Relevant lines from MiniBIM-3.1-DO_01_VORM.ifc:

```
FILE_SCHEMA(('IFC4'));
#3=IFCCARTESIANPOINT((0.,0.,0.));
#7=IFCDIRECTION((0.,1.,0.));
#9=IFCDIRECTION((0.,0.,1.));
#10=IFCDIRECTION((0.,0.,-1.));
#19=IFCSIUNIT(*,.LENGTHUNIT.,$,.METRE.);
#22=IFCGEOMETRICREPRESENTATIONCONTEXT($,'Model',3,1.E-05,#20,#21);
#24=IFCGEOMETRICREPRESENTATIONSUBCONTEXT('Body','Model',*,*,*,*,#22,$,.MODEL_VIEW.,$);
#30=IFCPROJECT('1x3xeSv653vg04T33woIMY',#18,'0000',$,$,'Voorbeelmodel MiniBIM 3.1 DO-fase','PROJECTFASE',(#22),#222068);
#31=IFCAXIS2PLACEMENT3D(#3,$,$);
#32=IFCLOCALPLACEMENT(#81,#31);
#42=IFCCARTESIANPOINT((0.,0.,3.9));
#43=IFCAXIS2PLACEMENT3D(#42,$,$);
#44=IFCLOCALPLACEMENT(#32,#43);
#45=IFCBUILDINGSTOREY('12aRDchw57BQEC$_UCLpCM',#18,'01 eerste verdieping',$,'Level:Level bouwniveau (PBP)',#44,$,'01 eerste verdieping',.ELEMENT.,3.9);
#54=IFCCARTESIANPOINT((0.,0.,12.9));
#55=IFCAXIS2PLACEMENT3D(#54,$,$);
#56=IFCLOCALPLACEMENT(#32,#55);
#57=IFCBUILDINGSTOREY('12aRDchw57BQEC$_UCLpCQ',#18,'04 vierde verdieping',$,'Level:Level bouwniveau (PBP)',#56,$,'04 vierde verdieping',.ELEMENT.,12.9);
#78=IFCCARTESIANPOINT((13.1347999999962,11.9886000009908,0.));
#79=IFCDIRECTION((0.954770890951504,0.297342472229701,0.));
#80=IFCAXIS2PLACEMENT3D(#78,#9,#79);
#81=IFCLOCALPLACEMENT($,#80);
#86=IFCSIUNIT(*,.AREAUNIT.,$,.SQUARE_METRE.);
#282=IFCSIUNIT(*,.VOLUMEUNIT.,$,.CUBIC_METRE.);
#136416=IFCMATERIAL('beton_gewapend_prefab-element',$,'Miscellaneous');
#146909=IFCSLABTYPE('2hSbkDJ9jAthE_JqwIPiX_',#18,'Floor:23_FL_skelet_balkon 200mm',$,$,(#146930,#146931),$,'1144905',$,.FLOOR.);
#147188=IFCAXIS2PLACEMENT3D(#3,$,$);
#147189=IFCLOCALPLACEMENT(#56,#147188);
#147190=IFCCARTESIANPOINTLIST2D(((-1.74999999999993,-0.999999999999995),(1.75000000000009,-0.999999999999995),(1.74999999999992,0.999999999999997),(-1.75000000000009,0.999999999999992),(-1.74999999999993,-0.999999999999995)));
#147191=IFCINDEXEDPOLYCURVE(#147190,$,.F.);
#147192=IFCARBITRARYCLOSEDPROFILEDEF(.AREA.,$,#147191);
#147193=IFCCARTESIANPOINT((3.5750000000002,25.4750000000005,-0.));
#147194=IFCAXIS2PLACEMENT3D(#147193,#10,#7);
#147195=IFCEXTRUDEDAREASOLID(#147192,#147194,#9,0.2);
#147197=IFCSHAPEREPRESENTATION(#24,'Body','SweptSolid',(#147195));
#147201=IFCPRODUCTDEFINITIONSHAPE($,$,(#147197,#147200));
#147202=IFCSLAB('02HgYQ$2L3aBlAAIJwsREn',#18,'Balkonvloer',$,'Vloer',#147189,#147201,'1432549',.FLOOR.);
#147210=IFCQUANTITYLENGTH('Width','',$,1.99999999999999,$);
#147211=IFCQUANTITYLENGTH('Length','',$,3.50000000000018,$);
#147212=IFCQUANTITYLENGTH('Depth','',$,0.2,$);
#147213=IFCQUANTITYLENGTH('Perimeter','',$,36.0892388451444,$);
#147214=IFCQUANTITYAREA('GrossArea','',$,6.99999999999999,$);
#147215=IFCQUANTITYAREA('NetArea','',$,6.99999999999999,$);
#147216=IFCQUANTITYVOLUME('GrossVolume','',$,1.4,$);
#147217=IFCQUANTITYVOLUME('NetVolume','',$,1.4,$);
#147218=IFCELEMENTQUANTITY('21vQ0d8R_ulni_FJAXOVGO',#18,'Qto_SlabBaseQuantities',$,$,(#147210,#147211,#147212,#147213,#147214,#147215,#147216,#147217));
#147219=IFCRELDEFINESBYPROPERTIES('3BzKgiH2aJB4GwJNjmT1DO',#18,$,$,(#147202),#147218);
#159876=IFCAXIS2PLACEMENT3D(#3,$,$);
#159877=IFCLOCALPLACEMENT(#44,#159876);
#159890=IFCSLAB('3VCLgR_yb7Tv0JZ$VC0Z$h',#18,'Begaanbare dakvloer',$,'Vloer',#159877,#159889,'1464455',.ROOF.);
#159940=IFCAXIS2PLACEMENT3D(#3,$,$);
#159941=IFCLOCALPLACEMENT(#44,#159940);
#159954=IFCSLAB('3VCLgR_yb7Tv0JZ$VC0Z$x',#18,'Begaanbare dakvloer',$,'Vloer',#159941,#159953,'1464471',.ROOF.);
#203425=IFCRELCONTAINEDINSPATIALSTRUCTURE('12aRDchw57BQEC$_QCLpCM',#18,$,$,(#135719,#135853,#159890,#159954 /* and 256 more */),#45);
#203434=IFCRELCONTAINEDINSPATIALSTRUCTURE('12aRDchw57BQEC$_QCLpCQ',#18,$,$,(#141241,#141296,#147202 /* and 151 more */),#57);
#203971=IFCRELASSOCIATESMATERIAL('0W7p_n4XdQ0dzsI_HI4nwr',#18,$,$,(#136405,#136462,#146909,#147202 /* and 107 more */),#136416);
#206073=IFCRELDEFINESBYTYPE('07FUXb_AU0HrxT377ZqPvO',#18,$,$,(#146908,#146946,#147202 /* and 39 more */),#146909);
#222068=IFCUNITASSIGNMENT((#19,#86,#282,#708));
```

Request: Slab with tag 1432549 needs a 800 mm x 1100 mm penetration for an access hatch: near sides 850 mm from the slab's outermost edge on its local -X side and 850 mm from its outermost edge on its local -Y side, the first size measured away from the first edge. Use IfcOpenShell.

```python
import numpy as np
import ifcopenshell
import ifcopenshell.api.feature
import ifcopenshell.api.geometry
import ifcopenshell.api.pset
import ifcopenshell.api.root
import ifcopenshell.geom
import ifcopenshell.util.element
import ifcopenshell.util.placement
import ifcopenshell.util.representation
import ifcopenshell.util.shape
import ifcopenshell.util.unit

model = ifcopenshell.open("MiniBIM-3.1-DO_01_VORM.ifc")
unit_scale = ifcopenshell.util.unit.calculate_unit_scale(model)
area_scale = ifcopenshell.util.unit.calculate_unit_scale(model, "AREAUNIT")
volume_scale = ifcopenshell.util.unit.calculate_unit_scale(model, "VOLUMEUNIT")
settings = ifcopenshell.geom.settings()


def volume(element):
    """Net volume in cubic metres, openings subtracted."""
    shape = ifcopenshell.geom.create_shape(settings, element)
    return ifcopenshell.util.shape.get_volume(shape.geometry)


slab = model.by_guid("02HgYQ$2L3aBlAAIJwsREn")
before = volume(slab)

# Extent in the slab's own axes, in metres. The edges named are its -X and -Y sides.
slab_shape = ifcopenshell.geom.create_shape(settings, slab)
vertices = ifcopenshell.util.shape.get_vertices(slab_shape.geometry)
x_min, y_min, bottom = vertices.min(axis=0)
top = vertices[:, 2].max()

opening = ifcopenshell.api.root.create_entity(model, ifc_class="IfcOpeningElement", name="Access hatch opening", predefined_type="OPENING")
context = ifcopenshell.util.representation.get_context(model, "Model", "Body", "MODEL_VIEW")
width, depth = 0.8, 1.1
outline = [(0.0, 0.0), (width, 0.0), (width, depth), (0.0, depth), (0.0, 0.0)]
# Overshoot both faces by 50 mm so the cut is clean.
shape = ifcopenshell.api.geometry.add_slab_representation(
    model, context=context, depth=top - bottom + 0.1, polyline=outline
)
ifcopenshell.api.geometry.assign_representation(model, product=opening, representation=shape)

matrix = ifcopenshell.util.placement.get_local_placement(slab.ObjectPlacement)
matrix[:, 3] = matrix @ np.append(np.array([x_min + 0.85, y_min + 0.85, bottom - 0.05]) / unit_scale, 1.0)
ifcopenshell.api.geometry.edit_object_placement(model, product=opening, matrix=matrix, is_si=False)
ifcopenshell.api.feature.add_feature(model, feature=opening, element=slab)

after = volume(slab)

# Update the slab's stored quantities.
qto = model.by_id(ifcopenshell.util.element.get_pset(slab, "Qto_SlabBaseQuantities", should_inherit=False)["id"])
ifcopenshell.api.pset.edit_qto(model, qto=qto, properties={
    "NetArea": after / (top - bottom) / area_scale,
    "NetVolume": after / volume_scale,
})

print(f"slab volume {before:.3f} -> {after:.3f} m3")

model.write("MiniBIM-3.1-DO_01_VORM_rev.ifc")
```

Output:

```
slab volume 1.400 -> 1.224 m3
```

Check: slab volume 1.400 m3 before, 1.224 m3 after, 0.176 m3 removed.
